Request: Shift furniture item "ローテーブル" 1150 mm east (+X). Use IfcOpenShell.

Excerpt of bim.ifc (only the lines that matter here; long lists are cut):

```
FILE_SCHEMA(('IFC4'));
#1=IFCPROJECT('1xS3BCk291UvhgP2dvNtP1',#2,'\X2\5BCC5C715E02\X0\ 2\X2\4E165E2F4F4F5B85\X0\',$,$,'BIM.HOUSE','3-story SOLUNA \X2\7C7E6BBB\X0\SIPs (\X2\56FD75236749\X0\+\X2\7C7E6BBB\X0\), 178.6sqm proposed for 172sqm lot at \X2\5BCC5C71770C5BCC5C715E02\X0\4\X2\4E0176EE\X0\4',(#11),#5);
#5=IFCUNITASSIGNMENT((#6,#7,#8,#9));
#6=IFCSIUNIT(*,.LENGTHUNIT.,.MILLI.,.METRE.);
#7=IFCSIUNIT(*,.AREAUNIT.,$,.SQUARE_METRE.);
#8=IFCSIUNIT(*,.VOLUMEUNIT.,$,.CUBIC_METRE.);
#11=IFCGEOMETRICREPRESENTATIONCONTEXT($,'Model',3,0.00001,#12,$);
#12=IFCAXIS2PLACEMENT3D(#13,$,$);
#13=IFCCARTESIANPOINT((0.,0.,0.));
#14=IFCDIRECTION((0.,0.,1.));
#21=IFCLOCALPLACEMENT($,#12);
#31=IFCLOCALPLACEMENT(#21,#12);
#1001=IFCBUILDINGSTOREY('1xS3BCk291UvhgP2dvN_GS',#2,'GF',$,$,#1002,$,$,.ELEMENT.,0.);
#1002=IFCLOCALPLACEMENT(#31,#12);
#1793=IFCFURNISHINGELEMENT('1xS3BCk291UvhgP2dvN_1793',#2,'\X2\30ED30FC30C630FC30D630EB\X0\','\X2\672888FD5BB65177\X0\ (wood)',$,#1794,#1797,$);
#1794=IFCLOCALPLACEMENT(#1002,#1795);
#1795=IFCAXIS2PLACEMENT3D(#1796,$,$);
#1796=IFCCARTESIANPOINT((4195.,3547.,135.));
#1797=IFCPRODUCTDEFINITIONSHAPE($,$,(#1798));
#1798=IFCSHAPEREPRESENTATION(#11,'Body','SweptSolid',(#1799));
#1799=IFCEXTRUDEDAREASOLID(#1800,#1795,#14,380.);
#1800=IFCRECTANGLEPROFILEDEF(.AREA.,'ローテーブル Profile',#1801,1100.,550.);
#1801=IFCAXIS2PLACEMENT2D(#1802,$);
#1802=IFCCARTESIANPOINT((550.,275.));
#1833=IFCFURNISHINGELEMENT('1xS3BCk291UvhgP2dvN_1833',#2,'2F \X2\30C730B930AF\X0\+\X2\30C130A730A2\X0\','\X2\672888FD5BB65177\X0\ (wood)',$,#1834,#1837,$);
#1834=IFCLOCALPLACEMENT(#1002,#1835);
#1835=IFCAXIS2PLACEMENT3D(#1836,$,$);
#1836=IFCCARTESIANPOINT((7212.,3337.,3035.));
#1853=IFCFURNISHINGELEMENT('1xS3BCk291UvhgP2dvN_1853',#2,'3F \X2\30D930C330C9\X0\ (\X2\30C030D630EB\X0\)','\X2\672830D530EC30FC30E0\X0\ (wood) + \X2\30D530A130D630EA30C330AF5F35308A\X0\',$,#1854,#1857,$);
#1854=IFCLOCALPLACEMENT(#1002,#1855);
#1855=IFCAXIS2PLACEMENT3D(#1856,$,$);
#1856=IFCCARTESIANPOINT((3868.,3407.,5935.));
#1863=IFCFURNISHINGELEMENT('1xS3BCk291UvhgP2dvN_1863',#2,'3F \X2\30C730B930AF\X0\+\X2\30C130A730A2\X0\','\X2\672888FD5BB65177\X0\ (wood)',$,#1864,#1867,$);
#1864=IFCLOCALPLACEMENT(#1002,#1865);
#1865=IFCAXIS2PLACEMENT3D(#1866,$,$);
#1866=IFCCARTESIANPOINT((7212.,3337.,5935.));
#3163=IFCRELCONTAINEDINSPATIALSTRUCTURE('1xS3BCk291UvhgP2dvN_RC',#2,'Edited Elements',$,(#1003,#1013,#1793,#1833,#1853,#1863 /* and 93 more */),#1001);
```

```python
import ifcopenshell
import ifcopenshell.api.geometry
import ifcopenshell.util.placement
import ifcopenshell.util.unit

model = ifcopenshell.open("bim.ifc")
unit_scale = ifcopenshell.util.unit.calculate_unit_scale(model)

item = model.by_guid("1xS3BCk291UvhgP2dvN_1793")
matrix = ifcopenshell.util.placement.get_local_placement(item.ObjectPlacement)
matrix[0, 3] += 1.15 / unit_scale
ifcopenshell.api.geometry.edit_object_placement(model, product=item, matrix=matrix, is_si=False)

print(ifcopenshell.util.placement.get_local_placement(item.ObjectPlacement).round(3) + 0.0)

model.write("bim-out.ifc")
```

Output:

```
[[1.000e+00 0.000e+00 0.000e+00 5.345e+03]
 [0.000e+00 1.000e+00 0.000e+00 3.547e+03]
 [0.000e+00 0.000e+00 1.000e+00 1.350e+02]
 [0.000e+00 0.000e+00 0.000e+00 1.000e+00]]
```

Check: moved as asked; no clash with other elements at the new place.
